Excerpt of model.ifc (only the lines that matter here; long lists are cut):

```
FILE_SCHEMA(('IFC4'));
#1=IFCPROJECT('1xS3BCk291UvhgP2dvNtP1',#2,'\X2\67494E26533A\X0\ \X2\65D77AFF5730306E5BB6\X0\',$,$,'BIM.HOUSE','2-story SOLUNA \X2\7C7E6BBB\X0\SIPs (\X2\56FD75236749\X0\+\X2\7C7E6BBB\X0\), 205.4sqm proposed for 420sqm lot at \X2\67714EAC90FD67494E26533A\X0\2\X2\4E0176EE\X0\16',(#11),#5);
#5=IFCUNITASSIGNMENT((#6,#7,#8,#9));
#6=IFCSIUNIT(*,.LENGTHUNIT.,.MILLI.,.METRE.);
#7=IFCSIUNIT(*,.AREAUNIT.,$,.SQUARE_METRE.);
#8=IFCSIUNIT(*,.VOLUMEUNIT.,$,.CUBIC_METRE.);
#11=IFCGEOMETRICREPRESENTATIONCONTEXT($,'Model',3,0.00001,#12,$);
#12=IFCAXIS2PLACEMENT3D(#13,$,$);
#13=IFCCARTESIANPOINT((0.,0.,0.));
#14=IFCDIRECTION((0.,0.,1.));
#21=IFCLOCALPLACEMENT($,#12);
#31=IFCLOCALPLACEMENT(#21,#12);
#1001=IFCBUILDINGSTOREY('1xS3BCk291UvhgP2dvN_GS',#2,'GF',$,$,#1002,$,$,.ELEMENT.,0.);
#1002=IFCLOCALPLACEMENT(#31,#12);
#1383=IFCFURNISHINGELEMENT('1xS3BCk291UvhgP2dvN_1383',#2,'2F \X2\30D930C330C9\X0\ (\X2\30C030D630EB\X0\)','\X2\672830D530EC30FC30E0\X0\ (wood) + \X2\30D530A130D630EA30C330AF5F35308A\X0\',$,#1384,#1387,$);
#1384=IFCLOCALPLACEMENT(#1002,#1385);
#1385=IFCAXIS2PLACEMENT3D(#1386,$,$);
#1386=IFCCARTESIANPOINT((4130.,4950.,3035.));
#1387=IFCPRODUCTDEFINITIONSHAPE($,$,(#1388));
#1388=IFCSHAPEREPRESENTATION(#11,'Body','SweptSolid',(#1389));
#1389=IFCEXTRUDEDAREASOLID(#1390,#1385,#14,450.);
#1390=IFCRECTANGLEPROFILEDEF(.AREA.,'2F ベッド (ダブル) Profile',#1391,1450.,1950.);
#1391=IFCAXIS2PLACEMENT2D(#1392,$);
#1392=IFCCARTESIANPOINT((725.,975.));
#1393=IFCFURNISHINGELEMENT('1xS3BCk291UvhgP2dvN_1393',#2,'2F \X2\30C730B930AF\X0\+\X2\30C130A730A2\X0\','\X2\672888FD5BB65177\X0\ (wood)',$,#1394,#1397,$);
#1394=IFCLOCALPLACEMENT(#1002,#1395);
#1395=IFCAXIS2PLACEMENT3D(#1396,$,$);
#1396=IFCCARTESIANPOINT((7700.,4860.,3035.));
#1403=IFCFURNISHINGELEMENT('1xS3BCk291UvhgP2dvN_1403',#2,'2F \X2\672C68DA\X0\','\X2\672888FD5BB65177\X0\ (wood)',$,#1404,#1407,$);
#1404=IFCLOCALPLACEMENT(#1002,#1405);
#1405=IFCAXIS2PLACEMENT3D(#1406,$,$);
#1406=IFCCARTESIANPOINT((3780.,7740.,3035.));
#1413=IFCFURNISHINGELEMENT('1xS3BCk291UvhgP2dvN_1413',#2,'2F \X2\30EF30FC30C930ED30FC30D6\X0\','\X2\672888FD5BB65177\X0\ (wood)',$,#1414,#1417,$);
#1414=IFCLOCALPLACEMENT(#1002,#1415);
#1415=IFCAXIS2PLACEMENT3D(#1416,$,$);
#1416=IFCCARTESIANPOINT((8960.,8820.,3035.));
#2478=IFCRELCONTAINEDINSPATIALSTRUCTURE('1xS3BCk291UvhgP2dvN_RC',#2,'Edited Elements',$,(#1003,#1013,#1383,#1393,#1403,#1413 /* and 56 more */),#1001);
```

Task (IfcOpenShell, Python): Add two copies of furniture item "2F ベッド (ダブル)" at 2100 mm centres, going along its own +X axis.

```python
import ifcopenshell
import ifcopenshell.api.geometry
import ifcopenshell.api.root
import ifcopenshell.util.element
import ifcopenshell.util.placement
import ifcopenshell.util.unit

model = ifcopenshell.open("model.ifc")
unit_scale = ifcopenshell.util.unit.calculate_unit_scale(model)


def reuse_history(source, copy):
    """copy_class also copies each property set's owner history, people and application; keep the originals."""
    for rel in copy.IsDefinedBy:
        if rel.is_a("IfcRelDefinesByProperties") and (history := rel.RelatingPropertyDefinition.OwnerHistory):
            rel.RelatingPropertyDefinition.OwnerHistory = source.OwnerHistory
            ifcopenshell.util.element.remove_deep2(model, history)


source = model.by_id(1383)
base = ifcopenshell.util.placement.get_local_placement(source.ObjectPlacement)
step = base[:3, 0] * 2.1 / unit_scale

for i in range(1, 3):
    copy = ifcopenshell.api.root.copy_class(model, product=source)
    copy.Representation = ifcopenshell.util.element.copy_deep(
        model, source.Representation, exclude=["IfcGeometricRepresentationContext", "IfcRepresentationMap"]
    )
    reuse_history(source, copy)
    matrix = base.copy()
    matrix[:3, 3] += i * step
    print("added at", matrix[:3, 3].round(3) + 0.0)
    ifcopenshell.api.geometry.edit_object_placement(model, product=copy, matrix=matrix, is_si=False)

model.write("model_edited.ifc")
```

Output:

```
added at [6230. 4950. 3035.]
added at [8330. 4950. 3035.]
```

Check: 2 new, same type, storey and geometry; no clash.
